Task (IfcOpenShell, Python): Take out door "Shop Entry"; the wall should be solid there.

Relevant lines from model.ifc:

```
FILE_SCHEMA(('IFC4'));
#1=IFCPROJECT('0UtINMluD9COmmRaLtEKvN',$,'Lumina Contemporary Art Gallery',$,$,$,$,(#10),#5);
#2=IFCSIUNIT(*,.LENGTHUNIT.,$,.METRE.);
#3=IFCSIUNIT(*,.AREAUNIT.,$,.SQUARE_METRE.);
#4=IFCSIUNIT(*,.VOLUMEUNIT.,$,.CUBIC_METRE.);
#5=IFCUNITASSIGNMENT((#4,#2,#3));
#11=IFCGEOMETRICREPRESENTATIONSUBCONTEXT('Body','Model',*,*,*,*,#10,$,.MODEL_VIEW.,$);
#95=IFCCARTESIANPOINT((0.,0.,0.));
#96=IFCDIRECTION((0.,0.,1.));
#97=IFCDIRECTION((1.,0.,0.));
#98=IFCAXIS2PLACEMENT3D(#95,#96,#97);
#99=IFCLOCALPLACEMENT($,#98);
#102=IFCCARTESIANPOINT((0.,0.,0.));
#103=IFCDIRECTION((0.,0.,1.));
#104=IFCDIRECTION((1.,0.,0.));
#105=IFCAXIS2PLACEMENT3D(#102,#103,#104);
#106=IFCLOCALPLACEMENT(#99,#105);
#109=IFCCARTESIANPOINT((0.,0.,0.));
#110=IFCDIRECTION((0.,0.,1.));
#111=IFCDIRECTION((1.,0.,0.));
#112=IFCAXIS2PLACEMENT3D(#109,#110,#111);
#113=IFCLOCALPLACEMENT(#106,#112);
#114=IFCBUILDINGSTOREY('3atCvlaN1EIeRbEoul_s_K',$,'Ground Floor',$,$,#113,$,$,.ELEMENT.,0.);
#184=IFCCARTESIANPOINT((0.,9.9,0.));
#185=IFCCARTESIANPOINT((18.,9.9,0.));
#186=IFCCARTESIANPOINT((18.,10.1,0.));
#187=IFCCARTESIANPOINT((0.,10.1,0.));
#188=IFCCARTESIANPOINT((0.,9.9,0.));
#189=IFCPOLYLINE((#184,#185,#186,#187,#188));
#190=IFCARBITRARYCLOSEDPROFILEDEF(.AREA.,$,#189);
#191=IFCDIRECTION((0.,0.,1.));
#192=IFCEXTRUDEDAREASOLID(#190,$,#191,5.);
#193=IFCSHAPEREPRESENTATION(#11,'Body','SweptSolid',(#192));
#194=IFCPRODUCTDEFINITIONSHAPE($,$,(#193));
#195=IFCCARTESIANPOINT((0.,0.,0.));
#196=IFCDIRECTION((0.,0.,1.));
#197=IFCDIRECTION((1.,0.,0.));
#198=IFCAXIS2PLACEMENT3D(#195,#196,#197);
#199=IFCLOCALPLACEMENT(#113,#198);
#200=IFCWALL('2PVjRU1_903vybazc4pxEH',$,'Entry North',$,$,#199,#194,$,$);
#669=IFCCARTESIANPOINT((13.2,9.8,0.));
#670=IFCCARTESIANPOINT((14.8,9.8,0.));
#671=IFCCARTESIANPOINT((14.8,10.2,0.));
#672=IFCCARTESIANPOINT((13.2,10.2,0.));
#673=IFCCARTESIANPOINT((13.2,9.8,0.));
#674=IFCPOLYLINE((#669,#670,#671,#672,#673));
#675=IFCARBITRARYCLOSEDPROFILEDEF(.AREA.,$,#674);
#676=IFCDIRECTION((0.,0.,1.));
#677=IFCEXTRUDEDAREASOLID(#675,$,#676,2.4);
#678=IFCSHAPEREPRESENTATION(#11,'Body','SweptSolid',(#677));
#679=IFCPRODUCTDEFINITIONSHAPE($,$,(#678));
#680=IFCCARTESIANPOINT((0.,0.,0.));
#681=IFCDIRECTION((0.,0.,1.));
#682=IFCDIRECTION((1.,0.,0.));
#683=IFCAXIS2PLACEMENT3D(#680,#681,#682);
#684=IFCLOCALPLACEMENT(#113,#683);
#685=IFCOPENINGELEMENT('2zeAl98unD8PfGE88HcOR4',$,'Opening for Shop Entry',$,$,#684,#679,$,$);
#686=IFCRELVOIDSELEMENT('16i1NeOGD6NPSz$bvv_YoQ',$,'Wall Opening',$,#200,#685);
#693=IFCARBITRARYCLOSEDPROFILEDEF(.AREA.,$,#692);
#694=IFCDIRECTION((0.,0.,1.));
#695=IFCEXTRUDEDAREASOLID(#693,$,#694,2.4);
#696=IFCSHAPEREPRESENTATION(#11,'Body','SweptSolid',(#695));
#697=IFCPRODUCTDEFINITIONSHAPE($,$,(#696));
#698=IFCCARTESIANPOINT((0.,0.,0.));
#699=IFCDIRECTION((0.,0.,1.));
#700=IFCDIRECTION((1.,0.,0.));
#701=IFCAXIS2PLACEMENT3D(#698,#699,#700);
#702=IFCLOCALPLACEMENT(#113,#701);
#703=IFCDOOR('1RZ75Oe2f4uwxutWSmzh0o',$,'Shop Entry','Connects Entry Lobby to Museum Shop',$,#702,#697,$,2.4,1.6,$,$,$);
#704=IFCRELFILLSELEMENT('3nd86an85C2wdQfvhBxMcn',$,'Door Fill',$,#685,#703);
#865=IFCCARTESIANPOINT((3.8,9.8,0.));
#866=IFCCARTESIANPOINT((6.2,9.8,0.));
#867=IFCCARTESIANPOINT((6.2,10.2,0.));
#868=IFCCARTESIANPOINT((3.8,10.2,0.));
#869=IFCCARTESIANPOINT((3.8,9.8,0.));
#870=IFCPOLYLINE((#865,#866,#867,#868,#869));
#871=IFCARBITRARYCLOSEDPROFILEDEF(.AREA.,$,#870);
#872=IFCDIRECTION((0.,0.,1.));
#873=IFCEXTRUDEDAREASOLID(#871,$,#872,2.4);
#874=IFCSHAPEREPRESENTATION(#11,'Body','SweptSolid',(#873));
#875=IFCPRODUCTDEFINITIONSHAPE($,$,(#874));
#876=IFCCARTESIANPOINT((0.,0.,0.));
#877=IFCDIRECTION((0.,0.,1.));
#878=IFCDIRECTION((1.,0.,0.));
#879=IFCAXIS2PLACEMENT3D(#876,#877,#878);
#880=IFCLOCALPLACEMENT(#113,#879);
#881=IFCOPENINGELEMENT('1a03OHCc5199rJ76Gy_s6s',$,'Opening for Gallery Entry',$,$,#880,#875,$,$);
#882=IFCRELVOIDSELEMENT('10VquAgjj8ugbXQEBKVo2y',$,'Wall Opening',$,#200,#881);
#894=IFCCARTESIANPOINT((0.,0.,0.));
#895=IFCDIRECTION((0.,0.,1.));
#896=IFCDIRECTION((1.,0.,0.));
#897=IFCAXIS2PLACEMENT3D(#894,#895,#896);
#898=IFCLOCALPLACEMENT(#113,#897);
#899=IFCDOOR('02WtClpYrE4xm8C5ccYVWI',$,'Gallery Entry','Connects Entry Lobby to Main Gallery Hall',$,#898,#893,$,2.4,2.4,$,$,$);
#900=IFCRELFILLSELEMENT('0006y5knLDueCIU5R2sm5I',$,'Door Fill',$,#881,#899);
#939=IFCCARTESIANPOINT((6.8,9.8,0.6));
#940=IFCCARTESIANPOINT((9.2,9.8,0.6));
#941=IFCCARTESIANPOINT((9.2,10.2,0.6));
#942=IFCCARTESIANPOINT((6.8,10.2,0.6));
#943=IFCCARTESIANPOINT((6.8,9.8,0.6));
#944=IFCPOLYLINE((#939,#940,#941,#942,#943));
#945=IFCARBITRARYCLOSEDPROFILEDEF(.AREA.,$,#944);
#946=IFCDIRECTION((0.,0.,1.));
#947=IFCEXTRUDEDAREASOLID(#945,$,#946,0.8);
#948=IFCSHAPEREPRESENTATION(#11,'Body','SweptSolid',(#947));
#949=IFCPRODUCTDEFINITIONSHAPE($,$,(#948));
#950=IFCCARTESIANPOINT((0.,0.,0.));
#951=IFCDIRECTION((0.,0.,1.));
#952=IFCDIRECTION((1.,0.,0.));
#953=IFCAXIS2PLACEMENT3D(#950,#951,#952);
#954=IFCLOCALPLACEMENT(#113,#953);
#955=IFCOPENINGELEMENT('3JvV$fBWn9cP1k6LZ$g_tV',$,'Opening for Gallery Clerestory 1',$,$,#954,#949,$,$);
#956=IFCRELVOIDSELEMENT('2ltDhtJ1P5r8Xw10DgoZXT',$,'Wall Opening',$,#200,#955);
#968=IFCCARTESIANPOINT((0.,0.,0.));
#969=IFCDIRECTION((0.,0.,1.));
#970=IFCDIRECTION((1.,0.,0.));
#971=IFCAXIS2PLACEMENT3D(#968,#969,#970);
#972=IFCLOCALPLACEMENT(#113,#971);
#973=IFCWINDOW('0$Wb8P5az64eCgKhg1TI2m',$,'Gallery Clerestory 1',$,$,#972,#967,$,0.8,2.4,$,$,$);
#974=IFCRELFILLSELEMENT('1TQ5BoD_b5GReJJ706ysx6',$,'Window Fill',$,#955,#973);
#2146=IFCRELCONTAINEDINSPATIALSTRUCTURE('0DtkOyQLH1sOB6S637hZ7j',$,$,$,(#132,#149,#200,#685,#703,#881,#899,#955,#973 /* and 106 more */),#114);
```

```python
import ifcopenshell
import ifcopenshell.api.feature
import ifcopenshell.api.root
import ifcopenshell.geom
import ifcopenshell.util.shape

model = ifcopenshell.open("model.ifc")
settings = ifcopenshell.geom.settings()


def volume(element):
    """Net volume in cubic metres, openings subtracted."""
    shape = ifcopenshell.geom.create_shape(settings, element)
    return ifcopenshell.util.shape.get_volume(shape.geometry)


door = model.by_guid("1RZ75Oe2f4uwxutWSmzh0o")
opening = door.FillsVoids[0].RelatingOpeningElement
wall = opening.VoidsElements[0].RelatingBuildingElement
before = volume(wall)

ifcopenshell.api.root.remove_product(model, product=door)
ifcopenshell.api.feature.remove_feature(model, feature=opening)

after = volume(wall)

print(f"wall volume {before:.3f} -> {after:.3f} m3")

model.write("model_v2.ifc")
```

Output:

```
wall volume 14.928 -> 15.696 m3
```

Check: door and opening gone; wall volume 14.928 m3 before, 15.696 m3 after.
